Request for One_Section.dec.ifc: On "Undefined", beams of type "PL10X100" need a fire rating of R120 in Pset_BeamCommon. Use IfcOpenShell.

First a look at what the model holds.

```python
import ifcopenshell
import ifcopenshell.util.element

model = ifcopenshell.open("One_Section.dec.ifc")
print(model.schema)
storey = next(s for s in model.by_type("IfcBuildingStorey") if s.Name == "Undefined")
beams = [e for e in ifcopenshell.util.element.get_decomposition(storey) if e.is_a("IfcBeam")]
seen = {}
for e in beams:
    element_type = ifcopenshell.util.element.get_type(e)
    key = (element_type.Name if element_type != e and element_type else None, ifcopenshell.util.element.get_pset(e, "Pset_BeamCommon", "FireRating"))
    seen[key] = seen.get(key, 0) + 1
for (name, value), count in sorted(seen.items(), key=str):
    print(count, "x", name, "|", value)
```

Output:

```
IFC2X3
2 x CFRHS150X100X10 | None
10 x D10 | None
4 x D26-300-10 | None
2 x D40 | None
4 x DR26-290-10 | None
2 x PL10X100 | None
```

```python
import ifcopenshell
import ifcopenshell.api.pset
import ifcopenshell.util.element

model = ifcopenshell.open("One_Section.dec.ifc")

storey = next(s for s in model.by_type("IfcBuildingStorey") if s.Name == "Undefined")
beams = [e for e in ifcopenshell.util.element.get_decomposition(storey) if e.is_a("IfcBeam")]

count = 0
for e in beams:
    element_type = ifcopenshell.util.element.get_type(e)
    if element_type in (None, e) or element_type.Name != "PL10X100":
        continue
    found = ifcopenshell.util.element.get_pset(e, "Pset_BeamCommon", should_inherit=False)
    if found:
        pset = model.by_id(found["id"])
        if len(ifcopenshell.util.element.get_elements_by_pset(pset)) > 1:
            pset = ifcopenshell.api.pset.unshare_pset(model, products=[e], pset=pset)[0]
    else:
        pset = ifcopenshell.api.pset.add_pset(model, product=e, name="Pset_BeamCommon")
    ifcopenshell.api.pset.edit_pset(model, pset=pset, properties={"FireRating": "R120"})
    count += 1

print(count, "beams updated")

model.write("One_Section.dec-out.ifc")
```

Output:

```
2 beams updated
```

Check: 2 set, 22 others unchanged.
